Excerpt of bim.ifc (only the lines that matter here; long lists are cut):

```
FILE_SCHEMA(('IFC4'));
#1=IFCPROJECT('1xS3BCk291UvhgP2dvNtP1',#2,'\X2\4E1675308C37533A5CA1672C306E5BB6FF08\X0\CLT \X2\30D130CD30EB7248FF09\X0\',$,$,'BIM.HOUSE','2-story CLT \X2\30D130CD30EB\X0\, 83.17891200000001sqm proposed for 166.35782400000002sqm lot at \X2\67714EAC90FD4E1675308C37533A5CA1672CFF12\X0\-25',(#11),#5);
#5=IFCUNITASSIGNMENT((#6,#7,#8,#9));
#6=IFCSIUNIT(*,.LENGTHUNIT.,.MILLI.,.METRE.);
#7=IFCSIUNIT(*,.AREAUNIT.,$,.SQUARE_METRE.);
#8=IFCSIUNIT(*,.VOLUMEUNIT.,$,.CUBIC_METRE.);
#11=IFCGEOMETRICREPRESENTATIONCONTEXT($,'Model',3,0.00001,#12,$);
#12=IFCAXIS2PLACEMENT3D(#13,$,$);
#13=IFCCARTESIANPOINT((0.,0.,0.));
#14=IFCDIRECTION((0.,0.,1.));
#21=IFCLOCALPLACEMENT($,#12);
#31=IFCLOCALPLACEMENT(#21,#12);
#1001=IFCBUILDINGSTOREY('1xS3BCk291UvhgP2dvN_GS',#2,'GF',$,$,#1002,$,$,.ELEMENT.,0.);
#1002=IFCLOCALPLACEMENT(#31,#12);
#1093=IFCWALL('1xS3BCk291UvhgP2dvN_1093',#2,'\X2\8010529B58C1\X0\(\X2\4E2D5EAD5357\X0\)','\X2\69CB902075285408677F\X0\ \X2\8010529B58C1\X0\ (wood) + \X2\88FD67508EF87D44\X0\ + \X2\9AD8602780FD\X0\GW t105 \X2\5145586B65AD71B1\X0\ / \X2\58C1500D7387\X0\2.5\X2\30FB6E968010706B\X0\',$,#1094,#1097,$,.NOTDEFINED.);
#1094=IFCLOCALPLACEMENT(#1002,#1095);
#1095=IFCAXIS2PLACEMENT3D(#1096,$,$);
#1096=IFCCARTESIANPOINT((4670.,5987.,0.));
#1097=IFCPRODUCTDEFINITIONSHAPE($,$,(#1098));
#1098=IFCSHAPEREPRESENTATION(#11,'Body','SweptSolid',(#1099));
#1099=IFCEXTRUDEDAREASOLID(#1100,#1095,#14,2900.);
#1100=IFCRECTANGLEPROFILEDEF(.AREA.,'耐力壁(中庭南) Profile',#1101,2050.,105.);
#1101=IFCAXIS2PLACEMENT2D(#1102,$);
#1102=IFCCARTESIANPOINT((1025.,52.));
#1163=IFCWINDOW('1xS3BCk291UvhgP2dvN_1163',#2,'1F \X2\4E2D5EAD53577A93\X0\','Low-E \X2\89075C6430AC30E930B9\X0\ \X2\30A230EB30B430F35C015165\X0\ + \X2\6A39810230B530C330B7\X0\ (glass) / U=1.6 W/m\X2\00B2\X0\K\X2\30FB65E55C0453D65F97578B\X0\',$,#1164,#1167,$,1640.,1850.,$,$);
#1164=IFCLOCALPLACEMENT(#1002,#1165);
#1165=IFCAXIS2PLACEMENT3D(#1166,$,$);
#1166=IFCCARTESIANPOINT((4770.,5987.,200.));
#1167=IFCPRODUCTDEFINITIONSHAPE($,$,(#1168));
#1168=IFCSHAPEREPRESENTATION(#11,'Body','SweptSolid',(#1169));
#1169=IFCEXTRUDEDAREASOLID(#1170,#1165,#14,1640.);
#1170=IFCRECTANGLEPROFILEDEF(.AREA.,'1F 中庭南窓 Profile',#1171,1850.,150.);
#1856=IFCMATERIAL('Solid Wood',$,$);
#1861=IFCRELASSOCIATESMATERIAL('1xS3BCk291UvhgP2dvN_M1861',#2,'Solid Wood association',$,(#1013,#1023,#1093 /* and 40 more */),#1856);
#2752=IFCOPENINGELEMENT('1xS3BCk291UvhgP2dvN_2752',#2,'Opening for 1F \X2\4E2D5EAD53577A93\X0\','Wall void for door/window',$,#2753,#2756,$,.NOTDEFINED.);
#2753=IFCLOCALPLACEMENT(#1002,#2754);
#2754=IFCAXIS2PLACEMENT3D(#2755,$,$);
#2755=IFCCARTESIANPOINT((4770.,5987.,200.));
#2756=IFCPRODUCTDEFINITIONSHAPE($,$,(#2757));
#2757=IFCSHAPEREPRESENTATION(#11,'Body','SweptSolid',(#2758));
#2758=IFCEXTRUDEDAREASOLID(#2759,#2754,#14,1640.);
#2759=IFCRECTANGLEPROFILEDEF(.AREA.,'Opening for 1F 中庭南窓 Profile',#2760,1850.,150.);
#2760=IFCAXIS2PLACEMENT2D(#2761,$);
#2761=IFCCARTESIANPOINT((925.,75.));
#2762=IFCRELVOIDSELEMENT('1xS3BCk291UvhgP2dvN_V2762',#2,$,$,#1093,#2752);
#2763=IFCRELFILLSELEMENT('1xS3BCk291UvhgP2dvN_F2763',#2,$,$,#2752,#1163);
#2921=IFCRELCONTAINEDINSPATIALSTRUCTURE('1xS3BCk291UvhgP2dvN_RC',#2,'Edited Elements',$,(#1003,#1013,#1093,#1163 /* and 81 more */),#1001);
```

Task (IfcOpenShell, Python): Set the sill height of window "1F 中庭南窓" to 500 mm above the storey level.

```python
import numpy as np
import ifcopenshell
import ifcopenshell.api.geometry
import ifcopenshell.geom
import ifcopenshell.util.element
import ifcopenshell.util.placement
import ifcopenshell.util.shape
import ifcopenshell.util.unit

model = ifcopenshell.open("bim.ifc")
unit_scale = ifcopenshell.util.unit.calculate_unit_scale(model)

window = model.by_id(1163)
opening = window.FillsVoids[0].RelatingOpeningElement
storey = ifcopenshell.util.element.get_container(window, ifc_class="IfcBuildingStorey")
level = ifcopenshell.util.placement.get_local_placement(storey.ObjectPlacement)[2, 3]

# The opening's origin need not be at the sill, so measure its lowest point.
shape = ifcopenshell.geom.create_shape(ifcopenshell.geom.settings(), opening)
bottom = ifcopenshell.util.shape.get_shape_bottom_elevation(shape, shape.geometry) / unit_scale
dz = level + 500.0 - bottom

shift = np.array([0.0, 0.0, dz])
# The window is not placed relative to its opening, so move both.
for product in (opening, window):
    matrix = ifcopenshell.util.placement.get_local_placement(product.ObjectPlacement)
    matrix[:3, 3] += shift
    ifcopenshell.api.geometry.edit_object_placement(model, product=product, matrix=matrix, is_si=False)

print(f"moved by {dz * unit_scale:+.3f} m")

model.write("bim-out.ifc")
```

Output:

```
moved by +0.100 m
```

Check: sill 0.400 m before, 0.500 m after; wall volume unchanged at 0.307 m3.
